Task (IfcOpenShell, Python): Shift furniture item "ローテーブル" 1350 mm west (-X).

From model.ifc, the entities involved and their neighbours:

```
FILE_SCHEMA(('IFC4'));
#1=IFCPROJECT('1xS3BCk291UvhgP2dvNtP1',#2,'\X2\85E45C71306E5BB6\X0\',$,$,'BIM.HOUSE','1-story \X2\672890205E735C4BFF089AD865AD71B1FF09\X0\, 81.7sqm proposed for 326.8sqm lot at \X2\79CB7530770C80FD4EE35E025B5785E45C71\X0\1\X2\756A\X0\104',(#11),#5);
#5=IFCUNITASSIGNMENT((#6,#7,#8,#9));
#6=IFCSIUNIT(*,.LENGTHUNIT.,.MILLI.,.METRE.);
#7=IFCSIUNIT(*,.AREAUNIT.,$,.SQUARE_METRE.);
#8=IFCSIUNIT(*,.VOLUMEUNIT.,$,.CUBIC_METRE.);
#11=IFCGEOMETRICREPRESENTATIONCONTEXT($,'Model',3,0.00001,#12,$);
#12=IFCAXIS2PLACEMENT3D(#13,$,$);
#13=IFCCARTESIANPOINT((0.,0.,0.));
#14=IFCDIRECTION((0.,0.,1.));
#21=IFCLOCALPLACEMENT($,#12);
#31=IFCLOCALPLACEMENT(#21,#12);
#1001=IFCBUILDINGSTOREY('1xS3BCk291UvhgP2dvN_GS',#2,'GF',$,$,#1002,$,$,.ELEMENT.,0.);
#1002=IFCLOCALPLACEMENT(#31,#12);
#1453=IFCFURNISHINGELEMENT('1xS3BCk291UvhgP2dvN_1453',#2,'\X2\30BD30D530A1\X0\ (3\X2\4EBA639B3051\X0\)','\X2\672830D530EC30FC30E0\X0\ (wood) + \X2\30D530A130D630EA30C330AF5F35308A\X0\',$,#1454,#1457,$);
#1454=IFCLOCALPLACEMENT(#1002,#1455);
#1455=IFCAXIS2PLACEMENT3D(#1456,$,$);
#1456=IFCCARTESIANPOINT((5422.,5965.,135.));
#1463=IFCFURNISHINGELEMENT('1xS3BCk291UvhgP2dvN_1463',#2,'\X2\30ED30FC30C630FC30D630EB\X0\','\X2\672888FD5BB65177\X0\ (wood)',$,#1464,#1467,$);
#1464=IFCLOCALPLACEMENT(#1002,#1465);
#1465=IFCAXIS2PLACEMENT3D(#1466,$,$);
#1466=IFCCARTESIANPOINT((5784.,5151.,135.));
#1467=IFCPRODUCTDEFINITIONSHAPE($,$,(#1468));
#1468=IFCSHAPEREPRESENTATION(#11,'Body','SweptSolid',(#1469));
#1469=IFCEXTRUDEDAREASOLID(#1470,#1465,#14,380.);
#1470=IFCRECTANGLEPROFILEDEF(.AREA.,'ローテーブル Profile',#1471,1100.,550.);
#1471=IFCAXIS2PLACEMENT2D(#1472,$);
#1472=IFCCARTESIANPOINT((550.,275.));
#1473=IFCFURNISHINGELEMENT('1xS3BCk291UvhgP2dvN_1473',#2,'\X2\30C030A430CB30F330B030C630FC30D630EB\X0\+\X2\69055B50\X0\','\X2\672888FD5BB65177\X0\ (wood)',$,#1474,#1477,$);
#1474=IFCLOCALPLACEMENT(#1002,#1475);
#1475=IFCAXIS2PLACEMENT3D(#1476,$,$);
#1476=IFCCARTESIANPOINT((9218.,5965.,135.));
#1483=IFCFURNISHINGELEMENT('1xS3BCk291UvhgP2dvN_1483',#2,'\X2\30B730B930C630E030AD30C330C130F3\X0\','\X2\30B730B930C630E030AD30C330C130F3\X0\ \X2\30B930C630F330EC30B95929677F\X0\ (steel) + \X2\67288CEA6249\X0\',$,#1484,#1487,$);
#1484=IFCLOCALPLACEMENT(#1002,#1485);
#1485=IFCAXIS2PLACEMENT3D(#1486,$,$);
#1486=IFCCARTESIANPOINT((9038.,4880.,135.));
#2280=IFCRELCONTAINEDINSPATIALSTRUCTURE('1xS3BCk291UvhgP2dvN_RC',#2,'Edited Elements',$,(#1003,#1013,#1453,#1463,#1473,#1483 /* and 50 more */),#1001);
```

```python
import ifcopenshell
import ifcopenshell.api.geometry
import ifcopenshell.util.placement
import ifcopenshell.util.unit

model = ifcopenshell.open("model.ifc")
unit_scale = ifcopenshell.util.unit.calculate_unit_scale(model)

item = model.by_id(1463)
matrix = ifcopenshell.util.placement.get_local_placement(item.ObjectPlacement)
matrix[0, 3] -= 1.35 / unit_scale
ifcopenshell.api.geometry.edit_object_placement(model, product=item, matrix=matrix, is_si=False)

print(ifcopenshell.util.placement.get_local_placement(item.ObjectPlacement).round(3) + 0.0)

model.write("model-out.ifc")
```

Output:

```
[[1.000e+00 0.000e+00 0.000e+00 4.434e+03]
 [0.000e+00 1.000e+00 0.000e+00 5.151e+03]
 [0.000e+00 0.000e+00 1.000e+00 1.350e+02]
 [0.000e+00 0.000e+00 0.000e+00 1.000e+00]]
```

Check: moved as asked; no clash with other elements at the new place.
